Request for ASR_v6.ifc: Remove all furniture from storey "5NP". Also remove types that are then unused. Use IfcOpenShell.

First a look at what the model holds.

```python
import ifcopenshell
import ifcopenshell.util.element

model = ifcopenshell.open("ASR_v6.ifc")
print(model.schema)
storey = next(s for s in model.by_type("IfcBuildingStorey") if s.Name == "5NP")
furniture = [e for e in ifcopenshell.util.element.get_decomposition(storey) if e.is_a("IfcFurnishingElement")]
seen = {}
for e in furniture:
    element_type = ifcopenshell.util.element.get_type(e)
    name = element_type.Name if element_type not in (None, e) else None
    seen[name] = seen.get(name, 0) + 1
for name, count in sorted(seen.items(), key=str):
    print(count, "x", name)
```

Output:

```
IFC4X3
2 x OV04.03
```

```python
import ifcopenshell
import ifcopenshell.api.root
import ifcopenshell.util.element

model = ifcopenshell.open("ASR_v6.ifc")

storey = next(s for s in model.by_type("IfcBuildingStorey") if s.Name == "5NP")
furniture = [e for e in ifcopenshell.util.element.get_decomposition(storey) if e.is_a("IfcFurnishingElement")]
types = {ifcopenshell.util.element.get_type(e) for e in furniture} - {None, *furniture}

for e in furniture:
    ifcopenshell.api.root.remove_product(model, product=e)
print(len(furniture), "removed")

unused = [t for t in types if not ifcopenshell.util.element.get_types(t)]
for t in unused:
    ifcopenshell.api.root.remove_product(model, product=t)
print(len(unused), "unused types removed")

model.write("ASR_v6-out.ifc")
```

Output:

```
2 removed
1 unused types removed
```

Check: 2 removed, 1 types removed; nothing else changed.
